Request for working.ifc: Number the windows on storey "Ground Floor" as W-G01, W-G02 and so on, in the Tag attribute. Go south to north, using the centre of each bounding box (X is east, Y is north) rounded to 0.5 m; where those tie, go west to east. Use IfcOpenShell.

First a look at what the model holds.

```python
import ifcopenshell
import ifcopenshell.util.element
import ifcopenshell.util.placement

model = ifcopenshell.open("working.ifc")
print(model.schema)
storey = next(s for s in model.by_type("IfcBuildingStorey") if s.Name == "Ground Floor")
windows = [e for e in ifcopenshell.util.element.get_decomposition(storey) if e.is_a("IfcWindow")]
for e in sorted(windows, key=lambda e: e.id()):
    origin = ifcopenshell.util.placement.get_local_placement(e.ObjectPlacement)[:3, 3]
    print(e.id(), e.Tag, e.Name, origin.round(2) + 0.0, sep=" | ")
```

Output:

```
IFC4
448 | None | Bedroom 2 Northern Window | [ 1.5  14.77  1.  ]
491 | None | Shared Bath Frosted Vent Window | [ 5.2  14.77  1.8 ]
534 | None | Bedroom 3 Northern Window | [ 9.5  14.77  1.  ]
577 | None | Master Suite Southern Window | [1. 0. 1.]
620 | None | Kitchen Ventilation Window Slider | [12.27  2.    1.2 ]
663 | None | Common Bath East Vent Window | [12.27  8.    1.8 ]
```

```python
import ifcopenshell
import ifcopenshell.geom
import ifcopenshell.util.element
import ifcopenshell.util.shape

model = ifcopenshell.open("working.ifc")
settings = ifcopenshell.geom.settings()
settings.set("use-world-coords", True)


def centre(element):
    shape = ifcopenshell.geom.create_shape(settings, element)
    return ifcopenshell.util.shape.get_bbox_centroid(shape.geometry)


storey = next(s for s in model.by_type("IfcBuildingStorey") if s.Name == "Ground Floor")
windows = [e for e in ifcopenshell.util.element.get_decomposition(storey) if e.is_a("IfcWindow")]

# Insertion points can sit at a corner or the storey origin, so sort by the geometry (in metres).
centres = {e: centre(e) for e in windows}
windows.sort(key=lambda e: (round(centres[e][1] / 0.5), centres[e][0]))

for i, e in enumerate(windows, start=1):
    number = f"W-G{i:02d}"
    e.Tag = number
    print(e.id(), number)

model.write("working_updated.ifc")
```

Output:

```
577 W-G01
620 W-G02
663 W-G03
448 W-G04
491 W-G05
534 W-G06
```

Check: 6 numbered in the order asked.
